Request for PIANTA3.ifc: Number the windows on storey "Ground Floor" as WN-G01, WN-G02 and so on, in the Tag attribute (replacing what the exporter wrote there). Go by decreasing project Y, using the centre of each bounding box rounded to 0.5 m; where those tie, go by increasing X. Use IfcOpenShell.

First a look at what the model holds.

```python
import ifcopenshell
import ifcopenshell.util.element
import ifcopenshell.util.placement

model = ifcopenshell.open("PIANTA3.ifc")
print(model.schema)
storey = next(s for s in model.by_type("IfcBuildingStorey") if s.Name == "Ground Floor")
windows = [e for e in ifcopenshell.util.element.get_decomposition(storey) if e.is_a("IfcWindow")]
for e in sorted(windows, key=lambda e: e.id()):
    origin = ifcopenshell.util.placement.get_local_placement(e.ObjectPlacement)[:3, 3]
    print(e.id(), e.Tag, e.Name, origin.round(2) + 0.0, sep=" | ")
```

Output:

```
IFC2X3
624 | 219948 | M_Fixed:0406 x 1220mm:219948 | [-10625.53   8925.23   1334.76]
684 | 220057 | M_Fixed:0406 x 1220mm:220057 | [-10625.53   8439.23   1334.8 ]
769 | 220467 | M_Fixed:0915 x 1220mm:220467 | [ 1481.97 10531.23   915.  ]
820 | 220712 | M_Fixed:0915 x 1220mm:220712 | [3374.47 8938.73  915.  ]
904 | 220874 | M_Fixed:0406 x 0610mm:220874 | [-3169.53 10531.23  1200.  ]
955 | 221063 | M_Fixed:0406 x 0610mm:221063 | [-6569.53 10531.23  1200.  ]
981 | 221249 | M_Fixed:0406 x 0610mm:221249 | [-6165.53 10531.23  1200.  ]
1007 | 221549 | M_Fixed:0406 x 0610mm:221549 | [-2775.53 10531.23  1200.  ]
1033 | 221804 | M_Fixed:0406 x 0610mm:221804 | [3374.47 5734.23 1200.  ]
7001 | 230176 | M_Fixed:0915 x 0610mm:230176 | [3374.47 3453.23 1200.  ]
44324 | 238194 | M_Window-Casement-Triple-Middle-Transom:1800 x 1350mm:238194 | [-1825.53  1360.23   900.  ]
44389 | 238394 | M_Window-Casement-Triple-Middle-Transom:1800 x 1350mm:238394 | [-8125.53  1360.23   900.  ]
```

```python
import ifcopenshell
import ifcopenshell.geom
import ifcopenshell.util.element
import ifcopenshell.util.shape

model = ifcopenshell.open("PIANTA3.ifc")
settings = ifcopenshell.geom.settings()
settings.set("use-world-coords", True)


def centre(element):
    shape = ifcopenshell.geom.create_shape(settings, element)
    return ifcopenshell.util.shape.get_bbox_centroid(shape.geometry)


storey = next(s for s in model.by_type("IfcBuildingStorey") if s.Name == "Ground Floor")
windows = [e for e in ifcopenshell.util.element.get_decomposition(storey) if e.is_a("IfcWindow")]

# Insertion points can sit at a corner or the storey origin, so sort by the geometry (in metres).
centres = {e: centre(e) for e in windows}
windows.sort(key=lambda e: (-round(centres[e][1] / 0.5), centres[e][0]))

for i, e in enumerate(windows, start=1):
    number = f"WN-G{i:02d}"
    e.Tag = number
    print(e.id(), number)

model.write("PIANTA3_updated.ifc")
```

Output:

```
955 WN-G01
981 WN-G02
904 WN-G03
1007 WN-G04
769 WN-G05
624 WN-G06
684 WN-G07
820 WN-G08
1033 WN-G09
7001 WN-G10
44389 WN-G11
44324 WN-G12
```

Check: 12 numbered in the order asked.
